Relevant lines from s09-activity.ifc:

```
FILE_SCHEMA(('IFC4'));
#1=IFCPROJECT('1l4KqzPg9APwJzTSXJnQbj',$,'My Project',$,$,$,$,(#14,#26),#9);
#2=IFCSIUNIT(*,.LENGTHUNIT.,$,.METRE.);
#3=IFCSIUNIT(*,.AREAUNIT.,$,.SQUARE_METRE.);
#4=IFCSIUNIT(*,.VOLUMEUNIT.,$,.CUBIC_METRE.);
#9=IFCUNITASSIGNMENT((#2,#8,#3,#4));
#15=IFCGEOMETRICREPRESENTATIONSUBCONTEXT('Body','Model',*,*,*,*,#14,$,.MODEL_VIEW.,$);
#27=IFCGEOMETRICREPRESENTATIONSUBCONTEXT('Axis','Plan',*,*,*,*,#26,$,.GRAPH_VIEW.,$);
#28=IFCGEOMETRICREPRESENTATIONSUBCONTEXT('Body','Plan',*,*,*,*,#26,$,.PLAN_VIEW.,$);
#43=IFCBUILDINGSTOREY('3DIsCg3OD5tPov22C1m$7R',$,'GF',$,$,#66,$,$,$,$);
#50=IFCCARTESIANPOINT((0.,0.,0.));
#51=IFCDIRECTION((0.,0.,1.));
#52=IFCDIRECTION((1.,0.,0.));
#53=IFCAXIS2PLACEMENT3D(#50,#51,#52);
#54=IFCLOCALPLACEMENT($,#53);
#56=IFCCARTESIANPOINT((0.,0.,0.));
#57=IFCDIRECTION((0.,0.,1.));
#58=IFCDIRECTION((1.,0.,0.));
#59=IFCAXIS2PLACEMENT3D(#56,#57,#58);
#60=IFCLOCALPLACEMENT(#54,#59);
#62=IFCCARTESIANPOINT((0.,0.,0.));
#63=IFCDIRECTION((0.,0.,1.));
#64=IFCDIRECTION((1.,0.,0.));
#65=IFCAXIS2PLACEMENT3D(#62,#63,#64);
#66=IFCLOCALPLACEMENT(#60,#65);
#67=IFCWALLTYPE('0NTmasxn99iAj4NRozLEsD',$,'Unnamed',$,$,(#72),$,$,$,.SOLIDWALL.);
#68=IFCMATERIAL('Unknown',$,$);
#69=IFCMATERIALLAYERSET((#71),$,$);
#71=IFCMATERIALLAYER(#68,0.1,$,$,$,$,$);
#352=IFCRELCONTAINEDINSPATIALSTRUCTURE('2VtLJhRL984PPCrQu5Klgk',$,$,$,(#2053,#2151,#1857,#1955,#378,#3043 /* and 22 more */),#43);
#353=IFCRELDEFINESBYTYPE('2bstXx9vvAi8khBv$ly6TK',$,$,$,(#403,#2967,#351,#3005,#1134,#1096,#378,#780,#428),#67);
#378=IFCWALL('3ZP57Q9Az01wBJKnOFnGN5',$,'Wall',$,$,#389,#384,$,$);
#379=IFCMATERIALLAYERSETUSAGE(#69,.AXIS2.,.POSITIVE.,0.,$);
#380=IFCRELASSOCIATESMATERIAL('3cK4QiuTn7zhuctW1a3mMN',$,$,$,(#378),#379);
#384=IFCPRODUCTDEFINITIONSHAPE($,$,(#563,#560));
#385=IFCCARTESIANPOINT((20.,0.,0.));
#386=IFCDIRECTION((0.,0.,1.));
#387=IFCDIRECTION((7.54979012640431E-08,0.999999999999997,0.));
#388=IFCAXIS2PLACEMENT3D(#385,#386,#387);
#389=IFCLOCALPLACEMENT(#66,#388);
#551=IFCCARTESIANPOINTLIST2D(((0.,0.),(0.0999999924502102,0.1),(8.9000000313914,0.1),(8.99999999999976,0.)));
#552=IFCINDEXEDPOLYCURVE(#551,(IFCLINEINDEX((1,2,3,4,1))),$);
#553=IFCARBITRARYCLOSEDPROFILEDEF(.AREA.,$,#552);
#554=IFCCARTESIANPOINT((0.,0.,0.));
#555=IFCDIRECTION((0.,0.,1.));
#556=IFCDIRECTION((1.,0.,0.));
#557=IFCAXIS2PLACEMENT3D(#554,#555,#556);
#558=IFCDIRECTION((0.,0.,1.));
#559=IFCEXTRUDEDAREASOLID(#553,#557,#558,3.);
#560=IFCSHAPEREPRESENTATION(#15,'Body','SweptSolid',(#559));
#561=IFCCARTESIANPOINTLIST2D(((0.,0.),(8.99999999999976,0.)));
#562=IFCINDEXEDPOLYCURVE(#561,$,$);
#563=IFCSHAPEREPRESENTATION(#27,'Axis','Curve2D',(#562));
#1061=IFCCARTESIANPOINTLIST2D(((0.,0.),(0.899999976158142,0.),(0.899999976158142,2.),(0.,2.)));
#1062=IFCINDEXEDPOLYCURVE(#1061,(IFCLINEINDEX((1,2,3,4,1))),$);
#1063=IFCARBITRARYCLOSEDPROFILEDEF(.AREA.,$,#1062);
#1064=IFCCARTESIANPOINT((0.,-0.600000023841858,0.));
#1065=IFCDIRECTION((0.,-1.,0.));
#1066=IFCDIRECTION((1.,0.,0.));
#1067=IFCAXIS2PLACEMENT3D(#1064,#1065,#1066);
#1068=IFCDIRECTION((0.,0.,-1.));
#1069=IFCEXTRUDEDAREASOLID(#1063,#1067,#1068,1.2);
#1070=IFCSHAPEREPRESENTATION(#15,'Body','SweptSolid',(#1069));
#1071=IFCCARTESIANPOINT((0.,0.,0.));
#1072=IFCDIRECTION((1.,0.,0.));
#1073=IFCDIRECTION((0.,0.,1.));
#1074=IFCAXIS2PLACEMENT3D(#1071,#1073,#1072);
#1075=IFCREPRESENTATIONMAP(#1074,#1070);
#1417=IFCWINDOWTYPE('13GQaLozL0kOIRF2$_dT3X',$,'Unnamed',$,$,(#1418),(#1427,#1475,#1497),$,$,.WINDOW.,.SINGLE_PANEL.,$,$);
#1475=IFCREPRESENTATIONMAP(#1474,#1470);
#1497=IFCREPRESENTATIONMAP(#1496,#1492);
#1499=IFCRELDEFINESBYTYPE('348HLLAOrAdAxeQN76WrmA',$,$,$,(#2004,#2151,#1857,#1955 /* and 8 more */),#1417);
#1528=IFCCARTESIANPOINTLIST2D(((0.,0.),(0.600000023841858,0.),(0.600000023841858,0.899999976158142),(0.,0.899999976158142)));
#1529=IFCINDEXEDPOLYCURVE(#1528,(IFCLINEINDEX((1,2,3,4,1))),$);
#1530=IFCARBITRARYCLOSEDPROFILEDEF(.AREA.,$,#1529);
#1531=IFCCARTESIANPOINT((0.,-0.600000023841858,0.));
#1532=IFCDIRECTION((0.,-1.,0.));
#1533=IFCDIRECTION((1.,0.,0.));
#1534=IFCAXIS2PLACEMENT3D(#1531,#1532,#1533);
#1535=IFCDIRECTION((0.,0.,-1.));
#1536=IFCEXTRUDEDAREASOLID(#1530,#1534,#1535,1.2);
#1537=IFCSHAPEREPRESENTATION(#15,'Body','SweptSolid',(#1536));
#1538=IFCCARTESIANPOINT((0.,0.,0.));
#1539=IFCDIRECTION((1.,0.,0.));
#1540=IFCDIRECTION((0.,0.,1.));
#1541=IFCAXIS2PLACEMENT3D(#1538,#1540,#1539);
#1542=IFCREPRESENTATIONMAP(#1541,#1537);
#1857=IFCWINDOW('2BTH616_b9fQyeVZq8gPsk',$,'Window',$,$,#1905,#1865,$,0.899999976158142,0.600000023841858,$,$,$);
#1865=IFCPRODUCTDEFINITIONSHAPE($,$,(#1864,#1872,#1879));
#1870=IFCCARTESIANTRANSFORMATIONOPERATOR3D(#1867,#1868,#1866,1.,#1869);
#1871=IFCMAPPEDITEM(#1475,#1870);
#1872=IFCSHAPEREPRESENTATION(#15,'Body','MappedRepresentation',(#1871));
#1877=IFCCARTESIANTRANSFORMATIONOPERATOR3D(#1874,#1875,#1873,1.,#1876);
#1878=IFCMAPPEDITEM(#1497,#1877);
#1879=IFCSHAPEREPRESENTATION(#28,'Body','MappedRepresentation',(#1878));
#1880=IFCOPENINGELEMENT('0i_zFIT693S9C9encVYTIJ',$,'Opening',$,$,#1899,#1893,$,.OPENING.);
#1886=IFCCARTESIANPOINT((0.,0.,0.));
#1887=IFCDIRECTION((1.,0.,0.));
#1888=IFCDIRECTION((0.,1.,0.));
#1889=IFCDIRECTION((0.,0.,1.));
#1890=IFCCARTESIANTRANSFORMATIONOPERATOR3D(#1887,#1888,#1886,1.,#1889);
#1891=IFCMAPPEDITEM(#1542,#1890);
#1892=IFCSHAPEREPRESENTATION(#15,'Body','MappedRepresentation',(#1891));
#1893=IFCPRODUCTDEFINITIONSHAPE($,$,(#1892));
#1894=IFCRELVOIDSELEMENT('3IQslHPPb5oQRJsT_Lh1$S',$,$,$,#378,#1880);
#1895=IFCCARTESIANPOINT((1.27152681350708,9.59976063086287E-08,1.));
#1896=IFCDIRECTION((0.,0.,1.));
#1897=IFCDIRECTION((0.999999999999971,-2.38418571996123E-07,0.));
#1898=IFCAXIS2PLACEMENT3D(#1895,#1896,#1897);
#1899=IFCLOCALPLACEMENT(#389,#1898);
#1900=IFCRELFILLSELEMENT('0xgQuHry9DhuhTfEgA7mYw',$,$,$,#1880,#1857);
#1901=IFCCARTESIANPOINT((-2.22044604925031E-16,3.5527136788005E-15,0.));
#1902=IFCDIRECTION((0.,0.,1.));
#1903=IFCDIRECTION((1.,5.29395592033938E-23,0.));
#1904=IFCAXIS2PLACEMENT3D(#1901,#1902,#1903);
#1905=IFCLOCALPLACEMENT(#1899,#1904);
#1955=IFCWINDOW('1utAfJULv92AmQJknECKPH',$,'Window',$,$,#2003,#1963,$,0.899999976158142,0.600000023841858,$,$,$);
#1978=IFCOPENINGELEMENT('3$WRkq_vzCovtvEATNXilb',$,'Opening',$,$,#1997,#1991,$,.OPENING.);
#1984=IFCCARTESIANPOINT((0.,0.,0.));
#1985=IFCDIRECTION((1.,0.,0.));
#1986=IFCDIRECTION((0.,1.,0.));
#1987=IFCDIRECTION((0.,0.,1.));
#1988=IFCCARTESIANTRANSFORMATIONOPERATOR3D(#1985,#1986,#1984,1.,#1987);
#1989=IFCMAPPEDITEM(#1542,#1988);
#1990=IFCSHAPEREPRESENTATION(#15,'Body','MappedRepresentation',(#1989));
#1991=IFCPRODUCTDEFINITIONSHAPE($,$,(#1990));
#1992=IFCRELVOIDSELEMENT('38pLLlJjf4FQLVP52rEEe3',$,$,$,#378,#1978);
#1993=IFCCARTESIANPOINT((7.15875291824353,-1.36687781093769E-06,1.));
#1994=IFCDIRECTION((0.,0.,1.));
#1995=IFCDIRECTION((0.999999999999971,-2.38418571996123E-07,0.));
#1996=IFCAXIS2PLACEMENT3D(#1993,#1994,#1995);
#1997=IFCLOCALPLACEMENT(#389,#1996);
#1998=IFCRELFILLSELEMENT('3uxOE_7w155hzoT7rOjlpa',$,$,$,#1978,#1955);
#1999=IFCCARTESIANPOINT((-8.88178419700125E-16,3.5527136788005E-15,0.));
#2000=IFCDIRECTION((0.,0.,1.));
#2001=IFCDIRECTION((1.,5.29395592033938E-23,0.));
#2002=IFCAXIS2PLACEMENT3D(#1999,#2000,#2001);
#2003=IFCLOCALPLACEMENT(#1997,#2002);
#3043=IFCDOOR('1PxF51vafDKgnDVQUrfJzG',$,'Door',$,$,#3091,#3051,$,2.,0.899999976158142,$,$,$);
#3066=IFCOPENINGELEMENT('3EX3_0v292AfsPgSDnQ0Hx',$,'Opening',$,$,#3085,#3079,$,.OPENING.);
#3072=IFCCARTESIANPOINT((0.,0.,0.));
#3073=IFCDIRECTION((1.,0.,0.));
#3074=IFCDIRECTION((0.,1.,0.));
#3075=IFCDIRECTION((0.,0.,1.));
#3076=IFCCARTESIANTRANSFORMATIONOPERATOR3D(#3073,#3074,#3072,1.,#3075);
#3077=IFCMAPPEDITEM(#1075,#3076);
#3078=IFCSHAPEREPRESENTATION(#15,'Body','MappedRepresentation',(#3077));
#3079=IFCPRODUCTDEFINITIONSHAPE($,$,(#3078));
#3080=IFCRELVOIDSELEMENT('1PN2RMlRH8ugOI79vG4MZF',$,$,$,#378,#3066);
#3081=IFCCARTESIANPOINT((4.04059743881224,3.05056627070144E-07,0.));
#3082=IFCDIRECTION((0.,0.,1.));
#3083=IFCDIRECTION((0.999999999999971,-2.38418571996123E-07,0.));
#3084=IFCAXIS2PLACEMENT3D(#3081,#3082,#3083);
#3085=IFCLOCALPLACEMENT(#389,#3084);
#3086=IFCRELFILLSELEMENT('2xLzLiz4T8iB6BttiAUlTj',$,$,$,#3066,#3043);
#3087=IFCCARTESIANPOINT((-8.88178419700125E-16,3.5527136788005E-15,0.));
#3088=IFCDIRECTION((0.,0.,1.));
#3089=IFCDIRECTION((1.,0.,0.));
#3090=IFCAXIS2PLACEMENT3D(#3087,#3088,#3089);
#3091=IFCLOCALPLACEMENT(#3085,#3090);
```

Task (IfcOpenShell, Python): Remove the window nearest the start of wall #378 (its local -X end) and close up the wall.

```python
import ifcopenshell
import ifcopenshell.api.feature
import ifcopenshell.api.root
import ifcopenshell.geom
import ifcopenshell.util.shape

model = ifcopenshell.open("s09-activity.ifc")
settings = ifcopenshell.geom.settings()


def volume(element):
    """Net volume in cubic metres, openings subtracted."""
    shape = ifcopenshell.geom.create_shape(settings, element)
    return ifcopenshell.util.shape.get_volume(shape.geometry)


window = model.by_guid("2BTH616_b9fQyeVZq8gPsk")
opening = window.FillsVoids[0].RelatingOpeningElement
wall = opening.VoidsElements[0].RelatingBuildingElement
before = volume(wall)

ifcopenshell.api.root.remove_product(model, product=window)
ifcopenshell.api.feature.remove_feature(model, feature=opening)

after = volume(wall)

print(f"wall volume {before:.3f} -> {after:.3f} m3")

model.write("s09-activity_v2.ifc")
```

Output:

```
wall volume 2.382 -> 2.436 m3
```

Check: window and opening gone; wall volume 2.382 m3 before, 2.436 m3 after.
